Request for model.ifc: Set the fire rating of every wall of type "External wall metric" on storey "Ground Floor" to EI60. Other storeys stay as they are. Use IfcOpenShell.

First a look at what the model holds.

```python
import ifcopenshell
import ifcopenshell.util.element

model = ifcopenshell.open("model.ifc")
print(model.schema)
storey = next(s for s in model.by_type("IfcBuildingStorey") if s.Name == "Ground Floor")
walls = [e for e in ifcopenshell.util.element.get_decomposition(storey) if e.is_a("IfcWall")]
seen = {}
for e in walls:
    element_type = ifcopenshell.util.element.get_type(e)
    key = (element_type.Name if element_type != e and element_type else None, ifcopenshell.util.element.get_pset(e, "Pset_WallCommon", "FireRating"))
    seen[key] = seen.get(key, 0) + 1
for (name, value), count in sorted(seen.items(), key=str):
    print(count, "x", name, "|", value)
```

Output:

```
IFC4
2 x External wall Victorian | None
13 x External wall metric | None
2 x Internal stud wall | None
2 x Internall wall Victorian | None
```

```python
import ifcopenshell
import ifcopenshell.api.pset
import ifcopenshell.util.element

model = ifcopenshell.open("model.ifc")

storey = next(s for s in model.by_type("IfcBuildingStorey") if s.Name == "Ground Floor")
walls = [e for e in ifcopenshell.util.element.get_decomposition(storey) if e.is_a("IfcWall")]

count = 0
for e in walls:
    element_type = ifcopenshell.util.element.get_type(e)
    if element_type in (None, e) or element_type.Name != "External wall metric":
        continue
    # add_pset returns the element's existing set when there is one.
    pset = ifcopenshell.api.pset.add_pset(model, product=e, name="Pset_WallCommon")
    ifcopenshell.api.pset.edit_pset(model, pset=pset, properties={"FireRating": "EI60"})
    count += 1

print(count, "walls updated")

model.write("model_v2.ifc")
```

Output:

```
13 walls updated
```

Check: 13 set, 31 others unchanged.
